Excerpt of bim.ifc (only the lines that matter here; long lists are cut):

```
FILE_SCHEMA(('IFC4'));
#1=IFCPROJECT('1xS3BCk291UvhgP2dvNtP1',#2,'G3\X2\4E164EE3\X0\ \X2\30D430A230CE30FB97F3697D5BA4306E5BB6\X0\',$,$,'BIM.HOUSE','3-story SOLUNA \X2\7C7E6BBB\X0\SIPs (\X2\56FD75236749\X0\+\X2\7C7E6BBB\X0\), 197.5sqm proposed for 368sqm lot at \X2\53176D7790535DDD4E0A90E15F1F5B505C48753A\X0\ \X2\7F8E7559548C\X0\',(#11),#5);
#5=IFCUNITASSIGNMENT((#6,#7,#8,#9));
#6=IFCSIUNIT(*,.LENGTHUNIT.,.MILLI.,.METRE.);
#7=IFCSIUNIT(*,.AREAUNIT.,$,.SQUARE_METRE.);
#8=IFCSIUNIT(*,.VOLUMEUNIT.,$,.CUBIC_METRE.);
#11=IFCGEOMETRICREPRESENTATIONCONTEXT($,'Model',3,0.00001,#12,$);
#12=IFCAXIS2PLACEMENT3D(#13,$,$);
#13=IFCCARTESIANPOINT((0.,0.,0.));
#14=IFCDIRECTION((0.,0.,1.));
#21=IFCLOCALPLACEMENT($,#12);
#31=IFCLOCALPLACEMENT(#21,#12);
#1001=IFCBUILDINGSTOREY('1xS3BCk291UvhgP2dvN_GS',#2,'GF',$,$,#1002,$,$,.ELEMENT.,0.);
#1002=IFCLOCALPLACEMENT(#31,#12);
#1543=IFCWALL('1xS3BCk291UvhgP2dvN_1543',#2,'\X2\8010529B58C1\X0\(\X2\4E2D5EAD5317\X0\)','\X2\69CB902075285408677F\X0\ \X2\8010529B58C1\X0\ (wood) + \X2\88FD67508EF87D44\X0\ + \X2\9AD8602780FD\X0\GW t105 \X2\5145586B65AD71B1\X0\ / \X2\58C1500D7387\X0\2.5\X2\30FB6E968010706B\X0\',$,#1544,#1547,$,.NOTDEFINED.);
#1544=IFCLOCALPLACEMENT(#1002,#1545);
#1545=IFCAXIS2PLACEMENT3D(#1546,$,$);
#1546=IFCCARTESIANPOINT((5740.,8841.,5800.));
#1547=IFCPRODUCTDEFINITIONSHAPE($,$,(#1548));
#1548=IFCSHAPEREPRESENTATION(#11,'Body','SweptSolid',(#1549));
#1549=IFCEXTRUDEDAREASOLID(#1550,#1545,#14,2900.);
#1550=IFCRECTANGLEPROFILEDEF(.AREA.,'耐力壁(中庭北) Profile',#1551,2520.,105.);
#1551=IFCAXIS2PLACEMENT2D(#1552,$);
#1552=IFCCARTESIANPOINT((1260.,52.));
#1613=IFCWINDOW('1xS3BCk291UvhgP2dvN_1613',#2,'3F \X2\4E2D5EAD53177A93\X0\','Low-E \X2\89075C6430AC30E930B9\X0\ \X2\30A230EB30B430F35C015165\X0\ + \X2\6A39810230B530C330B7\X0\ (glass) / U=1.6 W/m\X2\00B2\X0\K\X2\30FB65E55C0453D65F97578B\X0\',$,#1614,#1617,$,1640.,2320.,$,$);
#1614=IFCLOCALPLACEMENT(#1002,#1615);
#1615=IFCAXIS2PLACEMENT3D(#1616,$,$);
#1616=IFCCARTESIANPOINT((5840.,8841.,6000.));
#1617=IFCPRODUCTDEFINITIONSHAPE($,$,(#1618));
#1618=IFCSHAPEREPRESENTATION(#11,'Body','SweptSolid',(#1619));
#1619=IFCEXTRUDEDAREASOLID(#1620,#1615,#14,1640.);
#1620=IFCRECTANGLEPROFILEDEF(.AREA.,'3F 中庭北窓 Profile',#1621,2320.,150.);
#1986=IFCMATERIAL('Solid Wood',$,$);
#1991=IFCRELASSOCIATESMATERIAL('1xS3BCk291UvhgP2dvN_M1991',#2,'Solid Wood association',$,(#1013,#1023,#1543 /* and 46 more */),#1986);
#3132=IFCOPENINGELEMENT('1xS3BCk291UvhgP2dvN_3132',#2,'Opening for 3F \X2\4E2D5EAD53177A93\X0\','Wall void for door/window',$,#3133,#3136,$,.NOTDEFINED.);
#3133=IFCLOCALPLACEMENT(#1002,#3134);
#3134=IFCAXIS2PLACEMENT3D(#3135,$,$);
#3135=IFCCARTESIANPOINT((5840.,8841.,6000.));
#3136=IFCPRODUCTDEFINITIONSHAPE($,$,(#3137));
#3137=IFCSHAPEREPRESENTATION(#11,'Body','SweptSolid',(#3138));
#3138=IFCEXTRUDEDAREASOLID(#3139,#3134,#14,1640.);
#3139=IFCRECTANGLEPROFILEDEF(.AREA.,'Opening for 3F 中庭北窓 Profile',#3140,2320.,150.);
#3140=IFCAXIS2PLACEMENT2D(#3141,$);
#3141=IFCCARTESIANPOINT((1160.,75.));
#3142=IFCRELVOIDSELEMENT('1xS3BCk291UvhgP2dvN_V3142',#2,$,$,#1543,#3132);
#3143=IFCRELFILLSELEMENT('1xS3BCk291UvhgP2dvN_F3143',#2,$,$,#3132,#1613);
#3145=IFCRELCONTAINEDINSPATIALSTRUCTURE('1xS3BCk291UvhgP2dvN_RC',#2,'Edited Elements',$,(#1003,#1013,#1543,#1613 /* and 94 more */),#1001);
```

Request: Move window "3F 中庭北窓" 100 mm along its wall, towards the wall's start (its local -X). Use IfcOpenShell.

```python
import ifcopenshell
import ifcopenshell.api.geometry
import ifcopenshell.util.placement
import ifcopenshell.util.unit

model = ifcopenshell.open("bim.ifc")
unit_scale = ifcopenshell.util.unit.calculate_unit_scale(model)

window = model.by_guid("1xS3BCk291UvhgP2dvN_1613")
opening = window.FillsVoids[0].RelatingOpeningElement
wall = opening.VoidsElements[0].RelatingBuildingElement

wall_matrix = ifcopenshell.util.placement.get_local_placement(wall.ObjectPlacement)
shift = wall_matrix[:3, 0] * -0.1 / unit_scale
before = ifcopenshell.util.placement.get_local_placement(window.ObjectPlacement)[:3, 3].copy()

# The window is not placed relative to its opening, so move both.
for product in (opening, window):
    matrix = ifcopenshell.util.placement.get_local_placement(product.ObjectPlacement)
    matrix[:3, 3] += shift
    ifcopenshell.api.geometry.edit_object_placement(model, product=product, matrix=matrix, is_si=False)

after = ifcopenshell.util.placement.get_local_placement(window.ObjectPlacement)[:3, 3]
print("window moved by", (after - before).round(3) + 0.0)

model.write("bim_updated.ifc")
```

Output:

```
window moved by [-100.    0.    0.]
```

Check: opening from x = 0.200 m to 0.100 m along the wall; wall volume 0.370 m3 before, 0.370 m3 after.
